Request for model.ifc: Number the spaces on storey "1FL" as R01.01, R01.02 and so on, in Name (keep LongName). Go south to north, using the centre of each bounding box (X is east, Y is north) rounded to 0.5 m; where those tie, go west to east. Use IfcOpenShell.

First a look at what the model holds.

```python
import ifcopenshell
import ifcopenshell.util.element
import ifcopenshell.util.placement

model = ifcopenshell.open("model.ifc")
print(model.schema)
storey = next(s for s in model.by_type("IfcBuildingStorey") if s.Name == "1FL")
spaces = [e for e in ifcopenshell.util.element.get_decomposition(storey) if e.is_a("IfcSpace")]
for e in sorted(spaces, key=lambda e: e.id()):
    origin = ifcopenshell.util.placement.get_local_placement(e.ObjectPlacement)[:3, 3]
    print(e.id(), e.Name, e.LongName, origin.round(2) + 0.0, sep=" | ")
```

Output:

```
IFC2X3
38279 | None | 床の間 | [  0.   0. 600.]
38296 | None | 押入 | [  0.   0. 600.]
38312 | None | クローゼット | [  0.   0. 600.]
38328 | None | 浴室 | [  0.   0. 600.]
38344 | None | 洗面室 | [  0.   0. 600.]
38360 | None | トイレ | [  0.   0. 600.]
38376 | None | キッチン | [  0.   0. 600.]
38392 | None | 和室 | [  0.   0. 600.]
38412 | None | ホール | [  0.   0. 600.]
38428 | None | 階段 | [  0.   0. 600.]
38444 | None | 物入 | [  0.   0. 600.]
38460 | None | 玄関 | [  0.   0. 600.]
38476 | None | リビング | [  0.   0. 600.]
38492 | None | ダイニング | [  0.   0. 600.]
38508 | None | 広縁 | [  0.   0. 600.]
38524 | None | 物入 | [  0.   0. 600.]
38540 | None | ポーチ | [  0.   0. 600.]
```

```python
import ifcopenshell
import ifcopenshell.geom
import ifcopenshell.util.element
import ifcopenshell.util.shape

model = ifcopenshell.open("model.ifc")
settings = ifcopenshell.geom.settings()
settings.set("use-world-coords", True)


def centre(element):
    shape = ifcopenshell.geom.create_shape(settings, element)
    return ifcopenshell.util.shape.get_bbox_centroid(shape.geometry)


storey = next(s for s in model.by_type("IfcBuildingStorey") if s.Name == "1FL")
spaces = [e for e in ifcopenshell.util.element.get_decomposition(storey) if e.is_a("IfcSpace")]

# Insertion points can sit at a corner or the storey origin, so sort by the geometry (in metres).
centres = {e: centre(e) for e in spaces}
spaces.sort(key=lambda e: (round(centres[e][1] / 0.5), centres[e][0]))

for i, e in enumerate(spaces, start=1):
    number = f"R01.{i:02d}"
    e.Name = number
    print(e.id(), number)

model.write("model_v2.ifc")
```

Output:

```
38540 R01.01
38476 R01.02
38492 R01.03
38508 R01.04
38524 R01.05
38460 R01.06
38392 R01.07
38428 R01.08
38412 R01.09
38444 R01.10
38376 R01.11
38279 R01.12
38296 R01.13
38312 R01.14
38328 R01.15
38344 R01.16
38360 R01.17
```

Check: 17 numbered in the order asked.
